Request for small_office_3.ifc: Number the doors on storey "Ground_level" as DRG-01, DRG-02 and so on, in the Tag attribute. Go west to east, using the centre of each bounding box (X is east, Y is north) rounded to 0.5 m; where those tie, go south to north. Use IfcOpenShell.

First a look at what the model holds.

```python
import ifcopenshell
import ifcopenshell.util.element
import ifcopenshell.util.placement

model = ifcopenshell.open("small_office_3.ifc")
print(model.schema)
storey = next(s for s in model.by_type("IfcBuildingStorey") if s.Name == "Ground_level")
doors = [e for e in ifcopenshell.util.element.get_decomposition(storey) if e.is_a("IfcDoor")]
for e in sorted(doors, key=lambda e: e.id()):
    origin = ifcopenshell.util.placement.get_local_placement(e.ObjectPlacement)[:3, 3]
    print(e.id(), e.Tag, e.Name, origin.round(2) + 0.0, sep=" | ")
```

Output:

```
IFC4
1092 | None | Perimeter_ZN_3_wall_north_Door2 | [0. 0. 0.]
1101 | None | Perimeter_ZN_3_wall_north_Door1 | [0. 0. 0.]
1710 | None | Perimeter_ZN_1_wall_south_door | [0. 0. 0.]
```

```python
import ifcopenshell
import ifcopenshell.geom
import ifcopenshell.util.element
import ifcopenshell.util.shape

model = ifcopenshell.open("small_office_3.ifc")
settings = ifcopenshell.geom.settings()
settings.set("use-world-coords", True)


def centre(element):
    shape = ifcopenshell.geom.create_shape(settings, element)
    return ifcopenshell.util.shape.get_bbox_centroid(shape.geometry)


storey = next(s for s in model.by_type("IfcBuildingStorey") if s.Name == "Ground_level")
doors = [e for e in ifcopenshell.util.element.get_decomposition(storey) if e.is_a("IfcDoor")]

# Insertion points can sit at a corner or the storey origin, so sort by the geometry (in metres).
centres = {e: centre(e) for e in doors}
doors.sort(key=lambda e: (round(centres[e][0] / 0.5), centres[e][1]))

for i, e in enumerate(doors, start=1):
    number = f"DRG-{i:02d}"
    e.Tag = number
    print(e.id(), number)

model.write("small_office_3_edited.ifc")
```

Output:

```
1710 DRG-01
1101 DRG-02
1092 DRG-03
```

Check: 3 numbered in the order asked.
